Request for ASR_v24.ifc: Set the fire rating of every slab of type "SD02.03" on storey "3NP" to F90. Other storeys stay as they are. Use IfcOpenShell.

First a look at what the model holds.

```python
import ifcopenshell
import ifcopenshell.util.element

model = ifcopenshell.open("ASR_v24.ifc")
print(model.schema)
storey = next(s for s in model.by_type("IfcBuildingStorey") if s.Name == "3NP")
slabs = [e for e in ifcopenshell.util.element.get_decomposition(storey) if e.is_a("IfcSlab")]
seen = {}
for e in slabs:
    element_type = ifcopenshell.util.element.get_type(e)
    key = (element_type.Name if element_type != e and element_type else None, ifcopenshell.util.element.get_pset(e, "Pset_SlabCommon", "FireRating"))
    seen[key] = seen.get(key, 0) + 1
for (name, value), count in sorted(seen.items(), key=str):
    print(count, "x", name, "|", value)
```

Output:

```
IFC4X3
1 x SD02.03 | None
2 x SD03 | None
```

```python
import ifcopenshell
import ifcopenshell.api.pset
import ifcopenshell.util.element

model = ifcopenshell.open("ASR_v24.ifc")

storey = next(s for s in model.by_type("IfcBuildingStorey") if s.Name == "3NP")
slabs = [e for e in ifcopenshell.util.element.get_decomposition(storey) if e.is_a("IfcSlab")]

count = 0
for e in slabs:
    element_type = ifcopenshell.util.element.get_type(e)
    if element_type in (None, e) or element_type.Name != "SD02.03":
        continue
    # add_pset returns the element's existing set when there is one.
    pset = ifcopenshell.api.pset.add_pset(model, product=e, name="Pset_SlabCommon")
    ifcopenshell.api.pset.edit_pset(model, pset=pset, properties={"FireRating": "F90"})
    count += 1

print(count, "slabs updated")

model.write("ASR_v24_rev.ifc")
```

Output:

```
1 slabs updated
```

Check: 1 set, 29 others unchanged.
